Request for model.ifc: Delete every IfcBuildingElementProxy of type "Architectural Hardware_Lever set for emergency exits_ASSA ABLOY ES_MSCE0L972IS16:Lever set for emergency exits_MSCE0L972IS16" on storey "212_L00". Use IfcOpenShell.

First a look at what the model holds.

```python
import ifcopenshell
import ifcopenshell.util.element

model = ifcopenshell.open("model.ifc")
print(model.schema)
storey = next(s for s in model.by_type("IfcBuildingStorey") if s.Name == "212_L00")
proxies = [e for e in ifcopenshell.util.element.get_decomposition(storey) if e.is_a("IfcBuildingElementProxy")]
seen = {}
for e in proxies:
    element_type = ifcopenshell.util.element.get_type(e)
    name = element_type.Name if element_type not in (None, e) else None
    seen[name] = seen.get(name, 0) + 1
for name, count in sorted(seen.items(), key=str):
    print(count, "x", name)
```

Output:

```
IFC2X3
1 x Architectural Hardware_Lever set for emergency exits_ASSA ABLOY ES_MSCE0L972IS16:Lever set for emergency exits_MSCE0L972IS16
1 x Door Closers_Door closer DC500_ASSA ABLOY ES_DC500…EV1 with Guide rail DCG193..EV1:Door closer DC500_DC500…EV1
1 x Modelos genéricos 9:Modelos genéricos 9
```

```python
import ifcopenshell
import ifcopenshell.api.root
import ifcopenshell.util.element

model = ifcopenshell.open("model.ifc")

storey = next(s for s in model.by_type("IfcBuildingStorey") if s.Name == "212_L00")
proxies = [e for e in ifcopenshell.util.element.get_decomposition(storey) if e.is_a("IfcBuildingElementProxy")]
targets = [e for e in proxies if (t := ifcopenshell.util.element.get_type(e)) not in (None, e) and t.Name == "Architectural Hardware_Lever set for emergency exits_ASSA ABLOY ES_MSCE0L972IS16:Lever set for emergency exits_MSCE0L972IS16"]

for e in targets:
    ifcopenshell.api.root.remove_product(model, product=e)
print(len(targets), "removed")

model.write("model_rev.ifc")
```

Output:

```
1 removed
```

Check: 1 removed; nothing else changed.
